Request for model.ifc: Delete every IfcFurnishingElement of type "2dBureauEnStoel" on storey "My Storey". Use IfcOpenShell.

First a look at what the model holds.

```python
import ifcopenshell
import ifcopenshell.util.element

model = ifcopenshell.open("model.ifc")
print(model.schema)
storey = next(s for s in model.by_type("IfcBuildingStorey") if s.Name == "My Storey")
furniture = [e for e in ifcopenshell.util.element.get_decomposition(storey) if e.is_a("IfcFurnishingElement")]
seen = {}
for e in furniture:
    element_type = ifcopenshell.util.element.get_type(e)
    name = element_type.Name if element_type not in (None, e) else None
    seen[name] = seen.get(name, 0) + 1
for name, count in sorted(seen.items(), key=str):
    print(count, "x", name)
```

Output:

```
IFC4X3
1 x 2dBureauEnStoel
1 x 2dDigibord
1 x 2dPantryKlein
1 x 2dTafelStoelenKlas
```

```python
import ifcopenshell
import ifcopenshell.api.root
import ifcopenshell.util.element

model = ifcopenshell.open("model.ifc")

storey = next(s for s in model.by_type("IfcBuildingStorey") if s.Name == "My Storey")
furniture = [e for e in ifcopenshell.util.element.get_decomposition(storey) if e.is_a("IfcFurnishingElement")]
targets = [e for e in furniture if (t := ifcopenshell.util.element.get_type(e)) not in (None, e) and t.Name == "2dBureauEnStoel"]

for e in targets:
    ifcopenshell.api.root.remove_product(model, product=e)
print(len(targets), "removed")

model.write("model_edited.ifc")
```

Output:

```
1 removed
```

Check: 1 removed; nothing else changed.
